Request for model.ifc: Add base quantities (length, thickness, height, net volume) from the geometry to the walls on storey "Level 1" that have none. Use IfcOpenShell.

First a look at what the model holds.

```python
import ifcopenshell
import ifcopenshell.util.element
import ifcopenshell.util.unit

model = ifcopenshell.open("model.ifc")
print(model.schema)
for unit_type in ("LENGTHUNIT", "AREAUNIT", "VOLUMEUNIT"):
    print(unit_type, ifcopenshell.util.unit.calculate_unit_scale(model, unit_type))
storey = next(s for s in model.by_type("IfcBuildingStorey") if s.Name == "Level 1")
walls = [e for e in ifcopenshell.util.element.get_decomposition(storey) if e.is_a("IfcWall")]
for e in sorted(walls, key=lambda e: e.id()):
    print(e.id(), e.is_a(), e.Name, list(ifcopenshell.util.element.get_psets(e, qtos_only=True)), sep=" | ")
```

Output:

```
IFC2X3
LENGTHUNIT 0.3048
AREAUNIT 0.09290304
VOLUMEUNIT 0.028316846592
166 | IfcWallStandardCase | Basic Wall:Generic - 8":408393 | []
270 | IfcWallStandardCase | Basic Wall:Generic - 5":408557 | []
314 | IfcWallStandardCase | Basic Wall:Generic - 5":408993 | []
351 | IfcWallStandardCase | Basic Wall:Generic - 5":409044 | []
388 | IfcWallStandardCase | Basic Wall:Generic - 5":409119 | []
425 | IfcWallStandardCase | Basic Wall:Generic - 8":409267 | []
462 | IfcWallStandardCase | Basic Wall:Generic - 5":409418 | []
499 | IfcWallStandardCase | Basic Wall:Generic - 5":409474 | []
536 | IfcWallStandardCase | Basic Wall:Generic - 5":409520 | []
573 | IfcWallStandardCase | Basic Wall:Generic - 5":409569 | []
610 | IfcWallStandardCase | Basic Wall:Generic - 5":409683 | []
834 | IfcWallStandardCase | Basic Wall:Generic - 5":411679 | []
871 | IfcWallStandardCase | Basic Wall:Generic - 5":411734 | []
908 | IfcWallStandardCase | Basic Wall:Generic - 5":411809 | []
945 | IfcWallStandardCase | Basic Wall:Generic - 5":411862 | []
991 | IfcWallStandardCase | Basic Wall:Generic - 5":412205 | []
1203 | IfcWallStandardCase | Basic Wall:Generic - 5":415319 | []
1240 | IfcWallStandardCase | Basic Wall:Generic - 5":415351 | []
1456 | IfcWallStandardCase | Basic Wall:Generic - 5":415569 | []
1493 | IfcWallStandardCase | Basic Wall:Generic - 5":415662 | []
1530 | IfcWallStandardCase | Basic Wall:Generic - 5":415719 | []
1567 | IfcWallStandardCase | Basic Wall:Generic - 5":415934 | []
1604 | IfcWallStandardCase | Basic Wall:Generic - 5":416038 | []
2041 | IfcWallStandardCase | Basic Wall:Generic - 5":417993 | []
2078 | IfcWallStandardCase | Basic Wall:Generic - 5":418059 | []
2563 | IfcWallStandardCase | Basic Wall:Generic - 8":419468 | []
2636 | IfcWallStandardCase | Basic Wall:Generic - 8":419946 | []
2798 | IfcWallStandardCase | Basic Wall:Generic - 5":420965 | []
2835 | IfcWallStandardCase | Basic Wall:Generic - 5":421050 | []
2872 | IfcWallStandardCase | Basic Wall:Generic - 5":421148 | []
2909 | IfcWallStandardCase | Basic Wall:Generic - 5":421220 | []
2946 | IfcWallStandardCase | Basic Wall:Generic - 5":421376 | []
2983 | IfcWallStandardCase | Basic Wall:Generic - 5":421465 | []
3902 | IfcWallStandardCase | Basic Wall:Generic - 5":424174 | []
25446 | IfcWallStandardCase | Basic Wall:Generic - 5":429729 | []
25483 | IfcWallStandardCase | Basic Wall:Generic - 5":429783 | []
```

```python
import ifcopenshell
import ifcopenshell.api.pset
import ifcopenshell.geom
import ifcopenshell.util.element
import ifcopenshell.util.shape
import ifcopenshell.util.unit

model = ifcopenshell.open("model.ifc")
unit_scale = ifcopenshell.util.unit.calculate_unit_scale(model)
volume_scale = ifcopenshell.util.unit.calculate_unit_scale(model, "VOLUMEUNIT")
settings = ifcopenshell.geom.settings()

storey = next(s for s in model.by_type("IfcBuildingStorey") if s.Name == "Level 1")
walls = [e for e in ifcopenshell.util.element.get_decomposition(storey) if e.is_a("IfcWall")]

for e in sorted(walls, key=lambda e: e.id()):
    if ifcopenshell.util.element.get_psets(e, qtos_only=True, should_inherit=False):
        continue
    # Geometry comes back in metres, in the element's own axes.
    shape = ifcopenshell.geom.create_shape(settings, e)
    values = {
        "Length": ifcopenshell.util.shape.get_x(shape.geometry) / unit_scale,
        "Width": ifcopenshell.util.shape.get_y(shape.geometry) / unit_scale,
        "Height": ifcopenshell.util.shape.get_z(shape.geometry) / unit_scale,
        "NetVolume": ifcopenshell.util.shape.get_volume(shape.geometry) / volume_scale,
    }
    qto = ifcopenshell.api.pset.add_qto(model, product=e, name="BaseQuantities")
    ifcopenshell.api.pset.edit_qto(model, qto=qto, properties=values)
    print(e.id(), {k: round(v, 3) for k, v in values.items()})

model.write("model_updated.ifc")
```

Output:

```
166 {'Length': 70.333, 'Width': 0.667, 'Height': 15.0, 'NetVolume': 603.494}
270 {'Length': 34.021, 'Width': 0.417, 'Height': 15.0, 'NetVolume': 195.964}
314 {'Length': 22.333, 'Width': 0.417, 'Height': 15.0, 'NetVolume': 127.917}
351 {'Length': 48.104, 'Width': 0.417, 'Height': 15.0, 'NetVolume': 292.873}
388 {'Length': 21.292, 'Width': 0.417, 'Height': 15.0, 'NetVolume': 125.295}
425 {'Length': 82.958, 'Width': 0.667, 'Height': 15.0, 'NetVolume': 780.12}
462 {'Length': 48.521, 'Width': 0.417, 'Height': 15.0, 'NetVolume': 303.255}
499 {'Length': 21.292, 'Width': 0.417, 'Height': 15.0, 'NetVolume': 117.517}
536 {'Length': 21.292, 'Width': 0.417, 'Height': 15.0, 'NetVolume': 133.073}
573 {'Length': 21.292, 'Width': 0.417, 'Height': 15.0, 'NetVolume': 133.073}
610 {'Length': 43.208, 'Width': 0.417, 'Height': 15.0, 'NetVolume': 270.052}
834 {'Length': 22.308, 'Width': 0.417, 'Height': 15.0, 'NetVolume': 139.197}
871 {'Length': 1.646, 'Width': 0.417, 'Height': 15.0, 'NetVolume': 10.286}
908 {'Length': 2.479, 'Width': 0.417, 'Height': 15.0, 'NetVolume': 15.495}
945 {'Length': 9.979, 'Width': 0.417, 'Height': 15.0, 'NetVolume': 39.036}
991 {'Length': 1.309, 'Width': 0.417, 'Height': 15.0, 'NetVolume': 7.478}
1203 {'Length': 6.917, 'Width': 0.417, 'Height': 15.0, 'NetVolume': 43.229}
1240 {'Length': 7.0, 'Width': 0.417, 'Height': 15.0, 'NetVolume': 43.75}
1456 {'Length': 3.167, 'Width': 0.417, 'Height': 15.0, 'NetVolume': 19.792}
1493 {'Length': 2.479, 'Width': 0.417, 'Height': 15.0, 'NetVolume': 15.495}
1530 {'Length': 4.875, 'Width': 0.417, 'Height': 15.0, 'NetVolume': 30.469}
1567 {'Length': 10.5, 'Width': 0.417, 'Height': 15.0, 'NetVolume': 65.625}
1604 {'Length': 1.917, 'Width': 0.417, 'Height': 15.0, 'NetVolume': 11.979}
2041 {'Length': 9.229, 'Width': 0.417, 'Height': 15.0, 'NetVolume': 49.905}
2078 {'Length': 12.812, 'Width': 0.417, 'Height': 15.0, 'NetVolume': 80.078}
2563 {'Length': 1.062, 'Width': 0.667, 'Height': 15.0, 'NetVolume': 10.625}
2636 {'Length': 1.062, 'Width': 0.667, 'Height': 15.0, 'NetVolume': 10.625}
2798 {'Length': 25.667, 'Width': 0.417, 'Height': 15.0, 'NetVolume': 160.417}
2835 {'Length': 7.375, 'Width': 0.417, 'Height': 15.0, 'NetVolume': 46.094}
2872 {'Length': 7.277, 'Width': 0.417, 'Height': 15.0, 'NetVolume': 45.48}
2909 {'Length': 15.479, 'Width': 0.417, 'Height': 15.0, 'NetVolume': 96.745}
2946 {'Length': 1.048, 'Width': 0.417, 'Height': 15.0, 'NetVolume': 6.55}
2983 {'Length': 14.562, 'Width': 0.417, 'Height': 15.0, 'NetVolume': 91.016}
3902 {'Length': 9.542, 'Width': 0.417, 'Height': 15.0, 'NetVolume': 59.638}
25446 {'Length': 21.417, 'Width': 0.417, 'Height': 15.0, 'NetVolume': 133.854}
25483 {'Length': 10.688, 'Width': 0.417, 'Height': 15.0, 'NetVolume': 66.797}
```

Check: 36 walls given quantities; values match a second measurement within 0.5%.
